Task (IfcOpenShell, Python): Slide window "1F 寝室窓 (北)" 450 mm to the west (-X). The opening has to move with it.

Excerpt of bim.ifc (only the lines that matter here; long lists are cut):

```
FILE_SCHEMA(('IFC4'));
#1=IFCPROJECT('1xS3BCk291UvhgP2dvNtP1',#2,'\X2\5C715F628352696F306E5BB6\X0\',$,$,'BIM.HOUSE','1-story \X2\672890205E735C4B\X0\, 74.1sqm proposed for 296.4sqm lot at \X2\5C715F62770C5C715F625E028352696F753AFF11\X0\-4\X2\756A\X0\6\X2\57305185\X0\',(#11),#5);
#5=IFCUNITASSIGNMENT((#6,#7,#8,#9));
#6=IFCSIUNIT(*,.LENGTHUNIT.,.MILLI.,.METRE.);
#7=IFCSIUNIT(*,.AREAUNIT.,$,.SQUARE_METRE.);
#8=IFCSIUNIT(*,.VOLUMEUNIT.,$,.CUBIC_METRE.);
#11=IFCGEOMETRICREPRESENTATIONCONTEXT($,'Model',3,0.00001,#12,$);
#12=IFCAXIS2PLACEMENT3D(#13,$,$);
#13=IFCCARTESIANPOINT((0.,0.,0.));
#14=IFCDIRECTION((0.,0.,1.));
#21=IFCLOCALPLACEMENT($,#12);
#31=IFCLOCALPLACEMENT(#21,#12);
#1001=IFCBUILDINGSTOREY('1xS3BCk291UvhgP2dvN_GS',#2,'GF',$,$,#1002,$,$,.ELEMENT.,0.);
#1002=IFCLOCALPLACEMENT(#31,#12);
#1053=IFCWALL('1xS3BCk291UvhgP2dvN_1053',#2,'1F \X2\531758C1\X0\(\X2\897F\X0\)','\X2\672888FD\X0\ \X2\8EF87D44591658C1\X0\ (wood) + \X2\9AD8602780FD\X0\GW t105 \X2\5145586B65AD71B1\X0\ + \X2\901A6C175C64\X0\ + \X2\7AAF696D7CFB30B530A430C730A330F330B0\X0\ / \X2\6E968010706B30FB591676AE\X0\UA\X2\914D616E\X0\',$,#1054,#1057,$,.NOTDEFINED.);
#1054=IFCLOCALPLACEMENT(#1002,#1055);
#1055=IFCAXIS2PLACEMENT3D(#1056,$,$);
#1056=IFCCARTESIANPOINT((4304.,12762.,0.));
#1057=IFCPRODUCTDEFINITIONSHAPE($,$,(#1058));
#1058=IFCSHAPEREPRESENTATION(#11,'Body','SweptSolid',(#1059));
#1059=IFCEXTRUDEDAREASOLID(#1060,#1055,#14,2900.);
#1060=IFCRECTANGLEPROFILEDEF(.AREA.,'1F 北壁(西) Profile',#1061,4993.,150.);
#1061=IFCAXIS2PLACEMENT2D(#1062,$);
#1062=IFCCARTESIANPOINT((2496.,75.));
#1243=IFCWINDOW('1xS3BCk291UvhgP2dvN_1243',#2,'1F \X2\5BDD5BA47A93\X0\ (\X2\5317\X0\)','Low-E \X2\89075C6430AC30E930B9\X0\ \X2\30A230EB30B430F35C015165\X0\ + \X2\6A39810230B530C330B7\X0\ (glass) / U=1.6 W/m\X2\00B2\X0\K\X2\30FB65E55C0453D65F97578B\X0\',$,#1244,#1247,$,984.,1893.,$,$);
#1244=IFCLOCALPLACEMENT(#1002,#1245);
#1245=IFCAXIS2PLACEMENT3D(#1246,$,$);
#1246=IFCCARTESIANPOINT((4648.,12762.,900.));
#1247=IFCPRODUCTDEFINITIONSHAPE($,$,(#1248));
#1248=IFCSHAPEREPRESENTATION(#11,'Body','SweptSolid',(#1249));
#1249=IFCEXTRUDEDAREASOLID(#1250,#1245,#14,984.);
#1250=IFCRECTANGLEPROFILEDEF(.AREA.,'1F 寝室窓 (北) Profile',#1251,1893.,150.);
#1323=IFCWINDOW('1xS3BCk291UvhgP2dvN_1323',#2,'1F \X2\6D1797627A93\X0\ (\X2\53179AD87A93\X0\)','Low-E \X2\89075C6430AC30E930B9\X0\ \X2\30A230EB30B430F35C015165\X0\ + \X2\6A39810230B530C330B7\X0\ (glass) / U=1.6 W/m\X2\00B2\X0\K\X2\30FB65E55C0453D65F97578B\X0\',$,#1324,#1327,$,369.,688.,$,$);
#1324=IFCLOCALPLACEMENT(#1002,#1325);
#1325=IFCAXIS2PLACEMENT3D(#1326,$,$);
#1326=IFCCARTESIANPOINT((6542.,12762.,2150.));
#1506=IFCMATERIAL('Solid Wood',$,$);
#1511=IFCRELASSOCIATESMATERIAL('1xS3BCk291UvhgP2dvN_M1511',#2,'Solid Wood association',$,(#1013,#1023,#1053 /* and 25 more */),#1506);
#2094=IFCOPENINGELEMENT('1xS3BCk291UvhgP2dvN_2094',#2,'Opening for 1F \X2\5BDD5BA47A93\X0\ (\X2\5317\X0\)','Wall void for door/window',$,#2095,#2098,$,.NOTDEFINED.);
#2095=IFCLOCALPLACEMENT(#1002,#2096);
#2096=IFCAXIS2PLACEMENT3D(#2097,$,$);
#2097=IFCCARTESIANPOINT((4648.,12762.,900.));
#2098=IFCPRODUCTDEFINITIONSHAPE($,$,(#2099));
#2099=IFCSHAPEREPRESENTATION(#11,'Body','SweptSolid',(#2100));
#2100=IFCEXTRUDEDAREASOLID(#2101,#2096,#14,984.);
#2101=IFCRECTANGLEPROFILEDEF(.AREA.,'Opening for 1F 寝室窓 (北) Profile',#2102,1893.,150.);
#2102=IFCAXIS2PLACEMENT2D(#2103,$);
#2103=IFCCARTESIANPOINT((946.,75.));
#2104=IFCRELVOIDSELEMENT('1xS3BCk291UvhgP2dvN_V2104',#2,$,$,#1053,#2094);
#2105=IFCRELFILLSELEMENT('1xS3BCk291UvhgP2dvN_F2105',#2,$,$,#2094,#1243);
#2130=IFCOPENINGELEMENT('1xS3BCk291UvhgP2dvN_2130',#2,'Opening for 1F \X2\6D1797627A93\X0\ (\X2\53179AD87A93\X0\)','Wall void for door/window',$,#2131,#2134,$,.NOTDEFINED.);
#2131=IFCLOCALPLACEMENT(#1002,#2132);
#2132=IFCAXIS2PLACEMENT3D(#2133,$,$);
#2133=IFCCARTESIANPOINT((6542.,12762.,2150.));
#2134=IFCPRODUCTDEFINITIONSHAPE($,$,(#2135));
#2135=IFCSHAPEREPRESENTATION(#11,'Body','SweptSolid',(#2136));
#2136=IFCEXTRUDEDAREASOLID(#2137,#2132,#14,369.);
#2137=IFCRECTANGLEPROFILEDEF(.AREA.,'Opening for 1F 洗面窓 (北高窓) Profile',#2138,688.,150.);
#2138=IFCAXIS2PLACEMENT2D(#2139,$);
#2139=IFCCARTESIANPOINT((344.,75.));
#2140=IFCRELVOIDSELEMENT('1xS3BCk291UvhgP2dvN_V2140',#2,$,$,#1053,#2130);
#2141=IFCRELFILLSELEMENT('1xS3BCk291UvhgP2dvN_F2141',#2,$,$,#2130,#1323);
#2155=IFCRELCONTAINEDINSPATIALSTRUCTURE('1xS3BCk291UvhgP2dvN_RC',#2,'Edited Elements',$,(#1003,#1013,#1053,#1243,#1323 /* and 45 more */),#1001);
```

```python
import ifcopenshell
import ifcopenshell.api.geometry
import ifcopenshell.util.placement
import ifcopenshell.util.unit

model = ifcopenshell.open("bim.ifc")
unit_scale = ifcopenshell.util.unit.calculate_unit_scale(model)

window = model.by_guid("1xS3BCk291UvhgP2dvN_1243")
opening = window.FillsVoids[0].RelatingOpeningElement
wall = opening.VoidsElements[0].RelatingBuildingElement

wall_matrix = ifcopenshell.util.placement.get_local_placement(wall.ObjectPlacement)
shift = wall_matrix[:3, 0] * -0.45 / unit_scale
before = ifcopenshell.util.placement.get_local_placement(window.ObjectPlacement)[:3, 3].copy()

# The window is not placed relative to its opening, so move both.
for product in (opening, window):
    matrix = ifcopenshell.util.placement.get_local_placement(product.ObjectPlacement)
    matrix[:3, 3] += shift
    ifcopenshell.api.geometry.edit_object_placement(model, product=product, matrix=matrix, is_si=False)

after = ifcopenshell.util.placement.get_local_placement(window.ObjectPlacement)[:3, 3]
print("window moved by", (after - before).round(3) + 0.0)

model.write("bim_updated.ifc")
```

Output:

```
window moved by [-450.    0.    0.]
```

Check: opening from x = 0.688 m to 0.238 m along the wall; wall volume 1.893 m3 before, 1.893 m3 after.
